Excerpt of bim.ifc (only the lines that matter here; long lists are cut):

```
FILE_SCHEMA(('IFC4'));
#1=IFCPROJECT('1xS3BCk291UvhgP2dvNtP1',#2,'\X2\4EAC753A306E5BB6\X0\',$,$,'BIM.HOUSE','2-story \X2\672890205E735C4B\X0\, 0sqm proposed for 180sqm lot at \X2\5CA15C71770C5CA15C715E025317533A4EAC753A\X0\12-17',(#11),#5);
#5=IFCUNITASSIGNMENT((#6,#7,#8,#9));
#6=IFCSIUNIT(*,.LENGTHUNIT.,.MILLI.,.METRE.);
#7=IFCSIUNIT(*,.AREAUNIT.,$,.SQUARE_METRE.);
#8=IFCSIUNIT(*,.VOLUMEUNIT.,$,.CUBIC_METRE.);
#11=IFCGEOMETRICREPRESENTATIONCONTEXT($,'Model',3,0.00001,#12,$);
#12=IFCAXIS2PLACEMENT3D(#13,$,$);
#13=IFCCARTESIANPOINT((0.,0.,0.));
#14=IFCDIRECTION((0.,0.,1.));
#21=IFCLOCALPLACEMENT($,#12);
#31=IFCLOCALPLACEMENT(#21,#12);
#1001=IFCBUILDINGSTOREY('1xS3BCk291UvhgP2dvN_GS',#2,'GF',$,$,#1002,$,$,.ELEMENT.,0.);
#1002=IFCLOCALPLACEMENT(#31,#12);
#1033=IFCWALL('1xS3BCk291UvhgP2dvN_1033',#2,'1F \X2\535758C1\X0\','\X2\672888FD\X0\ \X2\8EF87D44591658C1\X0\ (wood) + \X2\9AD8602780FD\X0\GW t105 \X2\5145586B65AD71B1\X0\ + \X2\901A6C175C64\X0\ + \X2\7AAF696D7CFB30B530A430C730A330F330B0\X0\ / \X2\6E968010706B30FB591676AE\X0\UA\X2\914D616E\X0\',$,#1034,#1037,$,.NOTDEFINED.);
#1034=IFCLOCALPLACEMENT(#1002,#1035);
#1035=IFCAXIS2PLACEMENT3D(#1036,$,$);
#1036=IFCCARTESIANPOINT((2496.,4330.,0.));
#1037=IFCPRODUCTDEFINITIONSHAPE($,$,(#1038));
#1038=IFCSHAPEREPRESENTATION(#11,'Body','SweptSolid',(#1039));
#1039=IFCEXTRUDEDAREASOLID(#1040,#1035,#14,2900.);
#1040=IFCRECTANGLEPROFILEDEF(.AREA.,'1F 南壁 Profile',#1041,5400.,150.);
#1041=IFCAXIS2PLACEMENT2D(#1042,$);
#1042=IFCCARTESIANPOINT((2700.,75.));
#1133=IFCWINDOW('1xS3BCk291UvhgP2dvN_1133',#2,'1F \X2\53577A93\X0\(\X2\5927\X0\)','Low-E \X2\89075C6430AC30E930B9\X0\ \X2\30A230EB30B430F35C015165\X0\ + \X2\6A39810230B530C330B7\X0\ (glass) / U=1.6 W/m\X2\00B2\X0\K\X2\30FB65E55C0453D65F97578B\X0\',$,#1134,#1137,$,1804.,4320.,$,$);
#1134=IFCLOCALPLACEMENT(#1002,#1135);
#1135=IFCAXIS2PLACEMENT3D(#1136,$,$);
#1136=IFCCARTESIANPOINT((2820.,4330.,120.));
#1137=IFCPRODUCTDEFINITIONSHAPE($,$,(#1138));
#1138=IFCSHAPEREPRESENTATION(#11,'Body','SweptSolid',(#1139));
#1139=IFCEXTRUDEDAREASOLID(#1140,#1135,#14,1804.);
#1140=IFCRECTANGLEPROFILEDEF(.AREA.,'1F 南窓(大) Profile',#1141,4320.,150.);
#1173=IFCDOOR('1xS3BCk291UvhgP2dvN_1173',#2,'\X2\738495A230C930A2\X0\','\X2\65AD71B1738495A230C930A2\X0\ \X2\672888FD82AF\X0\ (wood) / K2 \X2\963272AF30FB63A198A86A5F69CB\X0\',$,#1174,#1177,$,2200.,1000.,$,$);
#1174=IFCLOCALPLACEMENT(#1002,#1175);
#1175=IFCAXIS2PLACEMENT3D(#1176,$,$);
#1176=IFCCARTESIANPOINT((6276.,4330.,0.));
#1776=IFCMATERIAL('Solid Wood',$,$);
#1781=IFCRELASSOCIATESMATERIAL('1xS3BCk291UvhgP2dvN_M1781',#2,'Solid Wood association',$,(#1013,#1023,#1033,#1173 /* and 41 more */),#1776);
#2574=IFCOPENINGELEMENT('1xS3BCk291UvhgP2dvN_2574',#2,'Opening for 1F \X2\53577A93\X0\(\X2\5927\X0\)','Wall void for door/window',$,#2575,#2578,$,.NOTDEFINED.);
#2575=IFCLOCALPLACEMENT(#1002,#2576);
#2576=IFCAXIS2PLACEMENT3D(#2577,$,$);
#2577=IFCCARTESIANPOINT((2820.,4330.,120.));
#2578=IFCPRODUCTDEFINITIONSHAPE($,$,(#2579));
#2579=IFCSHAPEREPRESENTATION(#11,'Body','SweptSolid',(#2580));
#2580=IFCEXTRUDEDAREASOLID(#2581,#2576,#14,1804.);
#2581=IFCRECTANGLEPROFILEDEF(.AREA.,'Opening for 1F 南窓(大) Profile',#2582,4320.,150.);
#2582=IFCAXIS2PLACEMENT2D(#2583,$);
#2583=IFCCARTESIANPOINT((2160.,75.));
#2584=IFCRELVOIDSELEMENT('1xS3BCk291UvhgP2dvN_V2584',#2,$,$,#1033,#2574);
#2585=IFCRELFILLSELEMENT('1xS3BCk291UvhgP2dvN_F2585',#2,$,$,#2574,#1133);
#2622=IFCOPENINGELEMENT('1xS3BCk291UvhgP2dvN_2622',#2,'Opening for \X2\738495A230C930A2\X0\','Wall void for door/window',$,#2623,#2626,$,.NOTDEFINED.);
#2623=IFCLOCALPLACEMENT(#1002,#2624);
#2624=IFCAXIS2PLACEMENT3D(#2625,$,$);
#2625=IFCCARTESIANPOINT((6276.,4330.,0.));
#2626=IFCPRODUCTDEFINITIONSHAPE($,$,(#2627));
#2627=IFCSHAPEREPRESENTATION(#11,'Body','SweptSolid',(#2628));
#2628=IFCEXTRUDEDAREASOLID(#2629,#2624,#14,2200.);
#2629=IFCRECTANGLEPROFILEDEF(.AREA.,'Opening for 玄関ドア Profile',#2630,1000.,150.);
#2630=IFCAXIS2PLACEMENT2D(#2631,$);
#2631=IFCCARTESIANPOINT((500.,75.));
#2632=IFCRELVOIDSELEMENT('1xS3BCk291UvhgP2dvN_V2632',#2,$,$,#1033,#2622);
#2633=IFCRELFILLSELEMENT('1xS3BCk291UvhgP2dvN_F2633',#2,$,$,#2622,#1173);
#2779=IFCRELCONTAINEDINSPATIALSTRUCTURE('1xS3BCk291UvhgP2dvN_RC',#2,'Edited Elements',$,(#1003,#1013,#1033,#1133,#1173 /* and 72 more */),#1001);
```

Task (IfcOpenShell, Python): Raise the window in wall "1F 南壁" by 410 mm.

```python
import numpy as np
import ifcopenshell
import ifcopenshell.api.geometry
import ifcopenshell.util.placement
import ifcopenshell.util.unit

model = ifcopenshell.open("bim.ifc")
unit_scale = ifcopenshell.util.unit.calculate_unit_scale(model)

window = model.by_id(1133)
opening = window.FillsVoids[0].RelatingOpeningElement
dz = 0.41 / unit_scale

shift = np.array([0.0, 0.0, dz])
# The window is not placed relative to its opening, so move both.
for product in (opening, window):
    matrix = ifcopenshell.util.placement.get_local_placement(product.ObjectPlacement)
    matrix[:3, 3] += shift
    ifcopenshell.api.geometry.edit_object_placement(model, product=product, matrix=matrix, is_si=False)

print(f"moved by {dz * unit_scale:+.3f} m")

model.write("bim_rev.ifc")
```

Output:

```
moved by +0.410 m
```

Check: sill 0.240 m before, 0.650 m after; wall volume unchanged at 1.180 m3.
